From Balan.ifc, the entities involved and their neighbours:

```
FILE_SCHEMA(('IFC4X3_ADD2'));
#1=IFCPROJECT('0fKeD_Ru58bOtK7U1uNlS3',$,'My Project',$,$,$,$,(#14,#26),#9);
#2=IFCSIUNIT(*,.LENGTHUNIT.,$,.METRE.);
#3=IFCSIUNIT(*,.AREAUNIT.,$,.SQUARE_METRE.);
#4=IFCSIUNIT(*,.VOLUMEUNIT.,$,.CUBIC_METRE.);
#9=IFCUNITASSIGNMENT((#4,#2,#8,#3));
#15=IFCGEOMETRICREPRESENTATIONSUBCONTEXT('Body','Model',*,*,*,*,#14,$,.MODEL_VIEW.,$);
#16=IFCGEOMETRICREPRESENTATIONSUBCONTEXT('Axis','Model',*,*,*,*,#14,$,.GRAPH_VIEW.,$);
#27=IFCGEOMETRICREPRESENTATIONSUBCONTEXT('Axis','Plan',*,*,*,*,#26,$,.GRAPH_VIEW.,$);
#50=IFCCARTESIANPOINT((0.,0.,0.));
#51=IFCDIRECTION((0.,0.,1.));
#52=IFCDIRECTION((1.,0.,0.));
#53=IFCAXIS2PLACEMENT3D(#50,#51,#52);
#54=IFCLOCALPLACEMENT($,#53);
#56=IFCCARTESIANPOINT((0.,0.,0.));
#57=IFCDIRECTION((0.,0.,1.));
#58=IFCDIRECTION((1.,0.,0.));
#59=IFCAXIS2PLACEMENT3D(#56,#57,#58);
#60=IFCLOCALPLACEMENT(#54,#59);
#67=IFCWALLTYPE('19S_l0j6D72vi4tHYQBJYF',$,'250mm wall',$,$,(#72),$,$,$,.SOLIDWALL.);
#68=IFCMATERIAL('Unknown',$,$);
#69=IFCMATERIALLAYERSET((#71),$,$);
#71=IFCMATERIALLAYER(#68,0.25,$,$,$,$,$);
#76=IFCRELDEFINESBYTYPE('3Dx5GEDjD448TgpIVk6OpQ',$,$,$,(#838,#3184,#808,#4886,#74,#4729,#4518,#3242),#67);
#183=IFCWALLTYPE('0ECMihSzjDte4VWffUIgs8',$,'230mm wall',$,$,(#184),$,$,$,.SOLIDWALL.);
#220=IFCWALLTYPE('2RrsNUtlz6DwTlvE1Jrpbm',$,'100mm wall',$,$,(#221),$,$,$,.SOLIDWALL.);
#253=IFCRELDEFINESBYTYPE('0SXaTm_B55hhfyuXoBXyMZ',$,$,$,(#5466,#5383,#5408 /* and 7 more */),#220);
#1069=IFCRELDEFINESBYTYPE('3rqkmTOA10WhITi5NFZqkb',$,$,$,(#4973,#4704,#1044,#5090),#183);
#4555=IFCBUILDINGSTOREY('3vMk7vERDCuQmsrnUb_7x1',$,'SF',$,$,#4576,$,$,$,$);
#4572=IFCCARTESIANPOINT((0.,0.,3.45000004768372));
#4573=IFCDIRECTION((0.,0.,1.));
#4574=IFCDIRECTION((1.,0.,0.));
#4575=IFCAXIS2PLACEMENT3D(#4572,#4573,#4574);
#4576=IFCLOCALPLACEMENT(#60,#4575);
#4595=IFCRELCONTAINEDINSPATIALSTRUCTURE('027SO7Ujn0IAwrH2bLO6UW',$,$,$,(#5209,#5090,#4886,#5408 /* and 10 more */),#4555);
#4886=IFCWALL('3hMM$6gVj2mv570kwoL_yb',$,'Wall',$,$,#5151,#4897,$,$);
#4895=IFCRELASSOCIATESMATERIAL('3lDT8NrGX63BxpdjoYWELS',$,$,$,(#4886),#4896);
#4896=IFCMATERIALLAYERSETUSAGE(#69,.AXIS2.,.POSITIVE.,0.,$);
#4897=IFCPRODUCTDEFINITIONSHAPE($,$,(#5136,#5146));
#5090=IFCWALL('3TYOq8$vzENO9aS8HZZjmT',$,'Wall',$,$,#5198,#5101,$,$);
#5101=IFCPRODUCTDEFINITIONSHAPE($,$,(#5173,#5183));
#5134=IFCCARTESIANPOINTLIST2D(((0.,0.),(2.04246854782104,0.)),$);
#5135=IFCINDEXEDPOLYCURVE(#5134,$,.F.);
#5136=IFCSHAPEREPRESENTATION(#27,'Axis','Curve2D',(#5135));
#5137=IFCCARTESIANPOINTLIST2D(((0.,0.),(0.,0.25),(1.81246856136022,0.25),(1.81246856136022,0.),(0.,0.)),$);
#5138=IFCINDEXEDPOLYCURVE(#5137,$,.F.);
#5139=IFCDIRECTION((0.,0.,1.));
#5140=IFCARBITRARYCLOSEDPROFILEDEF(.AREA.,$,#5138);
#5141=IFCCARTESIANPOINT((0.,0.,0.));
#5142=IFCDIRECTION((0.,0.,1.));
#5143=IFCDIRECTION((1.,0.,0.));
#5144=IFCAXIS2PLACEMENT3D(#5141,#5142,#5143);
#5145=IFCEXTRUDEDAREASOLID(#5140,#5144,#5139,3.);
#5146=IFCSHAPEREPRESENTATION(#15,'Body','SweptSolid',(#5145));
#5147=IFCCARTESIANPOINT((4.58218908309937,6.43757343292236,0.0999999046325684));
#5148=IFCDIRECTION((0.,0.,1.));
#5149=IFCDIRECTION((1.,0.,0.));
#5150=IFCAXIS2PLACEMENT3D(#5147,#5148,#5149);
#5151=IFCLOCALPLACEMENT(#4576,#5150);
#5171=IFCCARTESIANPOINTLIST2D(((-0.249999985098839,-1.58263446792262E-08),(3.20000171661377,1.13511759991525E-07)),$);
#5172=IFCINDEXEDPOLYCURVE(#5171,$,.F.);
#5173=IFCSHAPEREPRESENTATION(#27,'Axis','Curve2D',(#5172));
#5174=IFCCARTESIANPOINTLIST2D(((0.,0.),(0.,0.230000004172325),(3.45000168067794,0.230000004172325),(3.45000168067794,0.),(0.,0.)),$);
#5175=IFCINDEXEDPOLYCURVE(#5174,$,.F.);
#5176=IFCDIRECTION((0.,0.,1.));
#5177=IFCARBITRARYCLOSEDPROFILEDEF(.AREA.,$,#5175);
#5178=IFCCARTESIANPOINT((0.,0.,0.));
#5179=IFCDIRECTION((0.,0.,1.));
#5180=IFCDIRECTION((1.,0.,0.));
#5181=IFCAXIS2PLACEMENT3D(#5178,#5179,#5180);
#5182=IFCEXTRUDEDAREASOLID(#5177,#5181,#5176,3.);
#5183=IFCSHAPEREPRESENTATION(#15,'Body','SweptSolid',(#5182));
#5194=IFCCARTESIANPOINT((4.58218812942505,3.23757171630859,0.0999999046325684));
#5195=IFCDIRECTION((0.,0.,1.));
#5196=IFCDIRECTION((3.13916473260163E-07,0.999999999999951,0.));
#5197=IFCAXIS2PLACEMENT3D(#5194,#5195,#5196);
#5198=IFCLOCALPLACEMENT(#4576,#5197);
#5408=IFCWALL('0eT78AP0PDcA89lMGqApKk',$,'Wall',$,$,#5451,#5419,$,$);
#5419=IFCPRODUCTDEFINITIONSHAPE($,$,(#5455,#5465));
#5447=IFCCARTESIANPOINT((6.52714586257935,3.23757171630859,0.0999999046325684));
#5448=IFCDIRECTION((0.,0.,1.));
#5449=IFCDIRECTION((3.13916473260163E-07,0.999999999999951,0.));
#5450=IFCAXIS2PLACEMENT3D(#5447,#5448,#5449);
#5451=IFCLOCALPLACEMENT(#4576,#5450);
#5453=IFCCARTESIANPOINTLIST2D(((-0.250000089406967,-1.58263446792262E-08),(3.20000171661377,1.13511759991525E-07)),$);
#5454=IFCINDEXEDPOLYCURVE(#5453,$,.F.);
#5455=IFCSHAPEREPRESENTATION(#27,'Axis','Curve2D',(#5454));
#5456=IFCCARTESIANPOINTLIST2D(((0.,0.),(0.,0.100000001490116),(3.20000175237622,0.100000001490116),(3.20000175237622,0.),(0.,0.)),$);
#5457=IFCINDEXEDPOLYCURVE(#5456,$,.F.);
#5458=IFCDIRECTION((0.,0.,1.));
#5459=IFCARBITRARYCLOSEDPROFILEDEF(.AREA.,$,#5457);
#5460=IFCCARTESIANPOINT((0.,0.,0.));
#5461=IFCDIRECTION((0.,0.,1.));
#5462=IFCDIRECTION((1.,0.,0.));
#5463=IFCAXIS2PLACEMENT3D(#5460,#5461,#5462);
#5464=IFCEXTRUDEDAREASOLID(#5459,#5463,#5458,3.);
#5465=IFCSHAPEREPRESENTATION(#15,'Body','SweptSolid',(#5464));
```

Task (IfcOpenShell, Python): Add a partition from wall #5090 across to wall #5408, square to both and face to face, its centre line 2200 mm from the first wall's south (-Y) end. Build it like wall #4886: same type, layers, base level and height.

```python
import numpy as np
import ifcopenshell
import ifcopenshell.api.geometry
import ifcopenshell.api.material
import ifcopenshell.api.pset
import ifcopenshell.api.root
import ifcopenshell.api.spatial
import ifcopenshell.api.type
import ifcopenshell.geom
import ifcopenshell.util.element
import ifcopenshell.util.placement
import ifcopenshell.util.representation
import ifcopenshell.util.shape
import ifcopenshell.util.unit

model = ifcopenshell.open("Balan.ifc")
unit_scale = ifcopenshell.util.unit.calculate_unit_scale(model)
settings = ifcopenshell.geom.settings()
settings.set("use-world-coords", True)

start_wall = model.by_guid("3TYOq8$vzENO9aS8HZZjmT")
end_wall = model.by_guid("0eT78AP0PDcA89lMGqApKk")
like = model.by_guid("3hMM$6gVj2mv570kwoL_yb")
matrix = ifcopenshell.util.placement.get_local_placement(start_wall.ObjectPlacement)
matrix[:3, 3] *= unit_scale


def extent(element):
    """Bounding box in the first wall's axes, in metres."""
    shape = ifcopenshell.geom.create_shape(settings, element)
    points = (ifcopenshell.util.shape.get_vertices(shape.geometry) - matrix[:3, 3]) @ matrix[:3, :3]
    return points.min(axis=0), points.max(axis=0)


y_start = extent(start_wall)[0][1]
y_end = extent(end_wall)[1][1]
like_min, like_max = extent(like)
length, height = float(abs(y_end - y_start)), float(like_max[2] - like_min[2])
layer_set = ifcopenshell.util.element.get_material(like, should_skip_usage=True)
thickness = sum(layer.LayerThickness for layer in layer_set.MaterialLayers) * unit_scale

wall = ifcopenshell.api.root.create_entity(model, ifc_class="IfcWall", name="New partition")
storey = ifcopenshell.util.element.get_container(like)
ifcopenshell.api.spatial.assign_container(model, products=[wall], relating_structure=storey)
ifcopenshell.api.type.assign_type(
    model, related_objects=[wall], relating_type=ifcopenshell.util.element.get_type(like), should_map_representations=False
)
rel = ifcopenshell.api.material.assign_material(
    model, products=[wall], type="IfcMaterialLayerSetUsage", material=layer_set
)
rel.RelatingMaterial.OffsetFromReferenceLine = -thickness / 2 / unit_scale
pset = ifcopenshell.api.pset.add_pset(model, product=wall, name="Pset_WallCommon")
ifcopenshell.api.pset.edit_pset(model, pset=pset, properties={"IsExternal": False, "LoadBearing": False})

# The axis runs down the middle of the wall.
axis = ifcopenshell.api.geometry.add_axis_representation(
    model, context=ifcopenshell.util.representation.get_context(model, "Model", "Axis"), axis=[(0.0, 0.0), (length, 0.0)]
)
body = ifcopenshell.api.geometry.add_wall_representation(
    model,
    context=ifcopenshell.util.representation.get_context(model, "Model", "Body", "MODEL_VIEW"),
    length=length,
    height=height,
    thickness=thickness,
    offset=-thickness / 2,
)
for representation in (axis, body):
    ifcopenshell.api.geometry.assign_representation(model, product=wall, representation=representation)

placement = matrix @ ifcopenshell.util.placement.rotation(-90, "Z")
placement[:, 3] = matrix @ np.array([extent(start_wall)[0][0] + 2.2, y_start, like_min[2], 1.0])
ifcopenshell.api.geometry.edit_object_placement(model, product=wall, matrix=placement)

print(f"partition {length:.3f} m long, {height:.3f} m high, {thickness:.3f} m thick")

model.write("Balan_v2.ifc")
```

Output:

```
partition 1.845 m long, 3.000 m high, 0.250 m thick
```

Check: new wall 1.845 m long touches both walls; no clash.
